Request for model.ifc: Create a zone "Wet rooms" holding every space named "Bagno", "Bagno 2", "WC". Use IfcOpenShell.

First a look at what the model holds.

```python
import ifcopenshell

model = ifcopenshell.open("model.ifc")
print(model.schema)
seen = {}
for space in model.by_type("IfcSpace"):
    seen[space.LongName] = seen.get(space.LongName, 0) + 1
for name, count in sorted(seen.items(), key=str):
    print(count, "x", name)
print("zones:", [z.Name for z in model.by_type("IfcZone")][:20])
```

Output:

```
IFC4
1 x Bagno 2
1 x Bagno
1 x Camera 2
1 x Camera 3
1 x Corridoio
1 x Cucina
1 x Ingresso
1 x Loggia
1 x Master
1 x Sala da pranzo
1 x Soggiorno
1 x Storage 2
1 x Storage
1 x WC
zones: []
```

```python
import ifcopenshell
import ifcopenshell.api.group
import ifcopenshell.api.root

model = ifcopenshell.open("model.ifc")

names = {"Bagno", "Bagno 2", "WC"}
spaces = [s for s in model.by_type("IfcSpace") if s.LongName in names]

zone = ifcopenshell.api.root.create_entity(model, ifc_class="IfcZone", name="Wet rooms")
ifcopenshell.api.group.assign_group(model, products=spaces, group=zone)
print(len(spaces), "spaces in", zone.Name)

model.write("model_updated.ifc")
```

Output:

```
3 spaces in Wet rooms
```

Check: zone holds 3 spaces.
